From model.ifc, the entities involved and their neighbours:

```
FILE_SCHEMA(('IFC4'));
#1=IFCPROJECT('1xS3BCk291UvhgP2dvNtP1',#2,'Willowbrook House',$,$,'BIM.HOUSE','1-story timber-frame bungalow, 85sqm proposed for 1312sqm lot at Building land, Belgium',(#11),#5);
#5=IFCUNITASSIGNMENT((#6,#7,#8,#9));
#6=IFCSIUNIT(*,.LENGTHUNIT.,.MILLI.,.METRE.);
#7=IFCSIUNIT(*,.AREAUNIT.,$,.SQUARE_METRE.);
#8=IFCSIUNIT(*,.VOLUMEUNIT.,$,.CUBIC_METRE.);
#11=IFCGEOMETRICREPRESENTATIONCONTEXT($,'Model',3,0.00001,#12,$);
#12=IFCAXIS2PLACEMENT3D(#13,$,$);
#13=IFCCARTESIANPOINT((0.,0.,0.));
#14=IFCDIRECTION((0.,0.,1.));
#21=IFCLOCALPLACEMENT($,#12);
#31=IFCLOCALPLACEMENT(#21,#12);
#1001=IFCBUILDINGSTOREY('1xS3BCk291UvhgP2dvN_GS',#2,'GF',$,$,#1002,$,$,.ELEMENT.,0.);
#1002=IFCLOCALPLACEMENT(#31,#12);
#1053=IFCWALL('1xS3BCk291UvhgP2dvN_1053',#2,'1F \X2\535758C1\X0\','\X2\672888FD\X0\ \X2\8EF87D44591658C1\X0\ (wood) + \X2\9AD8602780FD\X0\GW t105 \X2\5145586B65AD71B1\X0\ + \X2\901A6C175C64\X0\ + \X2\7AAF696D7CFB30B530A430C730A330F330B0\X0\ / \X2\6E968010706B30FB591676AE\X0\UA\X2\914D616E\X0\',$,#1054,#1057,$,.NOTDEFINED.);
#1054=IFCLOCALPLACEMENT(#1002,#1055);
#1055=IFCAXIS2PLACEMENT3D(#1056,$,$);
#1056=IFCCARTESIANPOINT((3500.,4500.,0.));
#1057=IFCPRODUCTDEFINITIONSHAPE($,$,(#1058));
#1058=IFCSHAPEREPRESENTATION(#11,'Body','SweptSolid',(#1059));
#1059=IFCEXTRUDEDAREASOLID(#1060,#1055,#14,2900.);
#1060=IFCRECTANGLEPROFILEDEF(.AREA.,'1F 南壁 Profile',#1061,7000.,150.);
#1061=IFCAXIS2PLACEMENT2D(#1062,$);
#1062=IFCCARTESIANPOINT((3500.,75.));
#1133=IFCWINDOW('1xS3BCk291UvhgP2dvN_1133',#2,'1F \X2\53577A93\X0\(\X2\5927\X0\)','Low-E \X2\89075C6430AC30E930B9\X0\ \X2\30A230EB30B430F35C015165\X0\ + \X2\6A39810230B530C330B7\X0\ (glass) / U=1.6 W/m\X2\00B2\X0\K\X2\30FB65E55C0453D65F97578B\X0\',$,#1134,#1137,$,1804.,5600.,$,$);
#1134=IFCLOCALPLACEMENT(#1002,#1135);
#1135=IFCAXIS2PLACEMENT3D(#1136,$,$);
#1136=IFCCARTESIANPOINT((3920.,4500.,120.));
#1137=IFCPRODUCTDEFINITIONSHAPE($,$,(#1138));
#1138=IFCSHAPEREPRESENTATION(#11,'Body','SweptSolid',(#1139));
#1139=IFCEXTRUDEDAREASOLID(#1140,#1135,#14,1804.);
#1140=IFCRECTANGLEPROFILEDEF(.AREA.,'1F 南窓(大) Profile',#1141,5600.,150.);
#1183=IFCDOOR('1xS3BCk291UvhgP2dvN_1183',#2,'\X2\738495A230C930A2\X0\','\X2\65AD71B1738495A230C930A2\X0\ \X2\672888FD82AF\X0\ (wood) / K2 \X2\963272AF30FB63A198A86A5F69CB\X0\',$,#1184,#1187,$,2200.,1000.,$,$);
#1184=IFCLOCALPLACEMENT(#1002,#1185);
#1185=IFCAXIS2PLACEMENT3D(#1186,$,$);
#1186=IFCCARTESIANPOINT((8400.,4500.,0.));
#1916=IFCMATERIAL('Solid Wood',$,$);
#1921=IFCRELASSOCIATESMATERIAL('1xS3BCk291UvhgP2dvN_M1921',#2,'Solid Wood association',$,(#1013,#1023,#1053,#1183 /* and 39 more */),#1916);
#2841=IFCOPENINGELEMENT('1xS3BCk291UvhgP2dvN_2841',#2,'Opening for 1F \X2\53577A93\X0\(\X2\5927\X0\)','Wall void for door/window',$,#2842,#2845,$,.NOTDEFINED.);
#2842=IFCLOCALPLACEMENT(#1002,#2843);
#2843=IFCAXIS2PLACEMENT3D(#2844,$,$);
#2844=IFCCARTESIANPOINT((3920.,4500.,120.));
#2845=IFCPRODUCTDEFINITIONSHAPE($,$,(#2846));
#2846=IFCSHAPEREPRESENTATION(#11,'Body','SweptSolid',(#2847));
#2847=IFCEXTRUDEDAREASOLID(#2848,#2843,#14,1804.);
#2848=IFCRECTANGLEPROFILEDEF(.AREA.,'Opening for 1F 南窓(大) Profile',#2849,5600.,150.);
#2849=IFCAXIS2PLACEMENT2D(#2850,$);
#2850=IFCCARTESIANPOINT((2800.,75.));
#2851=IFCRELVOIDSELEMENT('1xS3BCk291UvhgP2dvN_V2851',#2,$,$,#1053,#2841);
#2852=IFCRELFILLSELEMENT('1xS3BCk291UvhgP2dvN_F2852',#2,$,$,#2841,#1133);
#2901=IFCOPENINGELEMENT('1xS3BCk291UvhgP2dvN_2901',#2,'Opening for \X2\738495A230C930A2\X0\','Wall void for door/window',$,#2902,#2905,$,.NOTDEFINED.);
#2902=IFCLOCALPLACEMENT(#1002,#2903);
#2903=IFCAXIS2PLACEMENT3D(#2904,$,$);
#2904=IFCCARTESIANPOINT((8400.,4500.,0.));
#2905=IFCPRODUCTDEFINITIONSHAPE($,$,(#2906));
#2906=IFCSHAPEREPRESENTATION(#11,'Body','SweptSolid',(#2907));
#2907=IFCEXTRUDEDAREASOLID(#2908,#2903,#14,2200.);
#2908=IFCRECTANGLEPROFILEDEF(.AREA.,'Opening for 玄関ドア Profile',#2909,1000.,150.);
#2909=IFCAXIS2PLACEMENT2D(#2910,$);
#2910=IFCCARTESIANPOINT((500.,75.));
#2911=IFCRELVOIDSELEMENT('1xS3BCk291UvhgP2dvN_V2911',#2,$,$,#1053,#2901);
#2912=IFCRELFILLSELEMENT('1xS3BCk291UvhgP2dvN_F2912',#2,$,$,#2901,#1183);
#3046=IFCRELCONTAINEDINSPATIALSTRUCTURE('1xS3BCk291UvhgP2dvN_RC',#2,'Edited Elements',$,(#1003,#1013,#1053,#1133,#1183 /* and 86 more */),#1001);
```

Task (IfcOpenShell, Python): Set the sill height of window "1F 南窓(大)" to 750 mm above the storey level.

```python
import numpy as np
import ifcopenshell
import ifcopenshell.api.geometry
import ifcopenshell.geom
import ifcopenshell.util.element
import ifcopenshell.util.placement
import ifcopenshell.util.shape
import ifcopenshell.util.unit

model = ifcopenshell.open("model.ifc")
unit_scale = ifcopenshell.util.unit.calculate_unit_scale(model)

window = model.by_guid("1xS3BCk291UvhgP2dvN_1133")
opening = window.FillsVoids[0].RelatingOpeningElement
storey = ifcopenshell.util.element.get_container(window, ifc_class="IfcBuildingStorey")
level = ifcopenshell.util.placement.get_local_placement(storey.ObjectPlacement)[2, 3]

# The opening's origin need not be at the sill, so measure its lowest point.
shape = ifcopenshell.geom.create_shape(ifcopenshell.geom.settings(), opening)
bottom = ifcopenshell.util.shape.get_shape_bottom_elevation(shape, shape.geometry) / unit_scale
dz = level + 0.75 / unit_scale - bottom

shift = np.array([0.0, 0.0, dz])
# The window is not placed relative to its opening, so move both.
for product in (opening, window):
    matrix = ifcopenshell.util.placement.get_local_placement(product.ObjectPlacement)
    matrix[:3, 3] += shift
    ifcopenshell.api.geometry.edit_object_placement(model, product=product, matrix=matrix, is_si=False)

print(f"moved by {dz * unit_scale:+.3f} m")

model.write("model-out.ifc")
```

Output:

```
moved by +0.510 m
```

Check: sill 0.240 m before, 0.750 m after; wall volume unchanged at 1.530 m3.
